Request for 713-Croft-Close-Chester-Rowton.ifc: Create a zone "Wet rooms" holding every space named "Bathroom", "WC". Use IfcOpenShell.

First a look at what the model holds.

```python
import ifcopenshell

model = ifcopenshell.open("713-Croft-Close-Chester-Rowton.ifc")
print(model.schema)
seen = {}
for space in model.by_type("IfcSpace"):
    seen[space.LongName] = seen.get(space.LongName, 0) + 1
for name, count in sorted(seen.items(), key=str):
    print(count, "x", name)
print("zones:", [z.Name for z in model.by_type("IfcZone")][:20])
```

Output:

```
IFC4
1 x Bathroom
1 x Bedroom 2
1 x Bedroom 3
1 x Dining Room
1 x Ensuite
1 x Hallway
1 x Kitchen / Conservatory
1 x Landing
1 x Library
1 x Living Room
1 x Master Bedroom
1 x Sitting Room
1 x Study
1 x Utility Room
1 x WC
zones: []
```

```python
import ifcopenshell
import ifcopenshell.api.group
import ifcopenshell.api.root

model = ifcopenshell.open("713-Croft-Close-Chester-Rowton.ifc")

names = {"Bathroom", "WC"}
spaces = [s for s in model.by_type("IfcSpace") if s.LongName in names]

zone = ifcopenshell.api.root.create_entity(model, ifc_class="IfcZone", name="Wet rooms")
ifcopenshell.api.group.assign_group(model, products=spaces, group=zone)
print(len(spaces), "spaces in", zone.Name)

model.write("713-Croft-Close-Chester-Rowton-out.ifc")
```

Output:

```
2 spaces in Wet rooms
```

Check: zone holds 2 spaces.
